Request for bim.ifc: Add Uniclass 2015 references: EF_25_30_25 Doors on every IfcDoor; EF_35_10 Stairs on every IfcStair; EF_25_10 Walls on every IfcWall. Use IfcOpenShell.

First a look at what the model holds.

```python
import ifcopenshell

model = ifcopenshell.open("bim.ifc")
print(model.schema)
print("classifications:", [c.Name for c in model.by_type("IfcClassification")])
for ifc_class in ("IfcDoor", "IfcRoof", "IfcStair", "IfcWall", "IfcWindow"):
    print(ifc_class, len(model.by_type(ifc_class)))
```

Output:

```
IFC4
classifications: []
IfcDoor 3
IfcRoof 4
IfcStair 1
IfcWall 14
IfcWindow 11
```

```python
import ifcopenshell
import ifcopenshell.api.classification

model = ifcopenshell.open("bim.ifc")

system = ifcopenshell.api.classification.add_classification(model, classification="Uniclass 2015")

codes = {
    "IfcDoor": ("EF_25_30_25", "Doors"),
    "IfcStair": ("EF_35_10", "Stairs"),
    "IfcWall": ("EF_25_10", "Walls"),
}
for ifc_class, (code, name) in codes.items():
    products = model.by_type(ifc_class)
    ifcopenshell.api.classification.add_reference(
        model, products=products, classification=system, identification=code, name=name
    )
    print(code, len(products))

model.write("bim_updated.ifc")
```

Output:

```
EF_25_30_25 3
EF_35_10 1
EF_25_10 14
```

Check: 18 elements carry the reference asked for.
